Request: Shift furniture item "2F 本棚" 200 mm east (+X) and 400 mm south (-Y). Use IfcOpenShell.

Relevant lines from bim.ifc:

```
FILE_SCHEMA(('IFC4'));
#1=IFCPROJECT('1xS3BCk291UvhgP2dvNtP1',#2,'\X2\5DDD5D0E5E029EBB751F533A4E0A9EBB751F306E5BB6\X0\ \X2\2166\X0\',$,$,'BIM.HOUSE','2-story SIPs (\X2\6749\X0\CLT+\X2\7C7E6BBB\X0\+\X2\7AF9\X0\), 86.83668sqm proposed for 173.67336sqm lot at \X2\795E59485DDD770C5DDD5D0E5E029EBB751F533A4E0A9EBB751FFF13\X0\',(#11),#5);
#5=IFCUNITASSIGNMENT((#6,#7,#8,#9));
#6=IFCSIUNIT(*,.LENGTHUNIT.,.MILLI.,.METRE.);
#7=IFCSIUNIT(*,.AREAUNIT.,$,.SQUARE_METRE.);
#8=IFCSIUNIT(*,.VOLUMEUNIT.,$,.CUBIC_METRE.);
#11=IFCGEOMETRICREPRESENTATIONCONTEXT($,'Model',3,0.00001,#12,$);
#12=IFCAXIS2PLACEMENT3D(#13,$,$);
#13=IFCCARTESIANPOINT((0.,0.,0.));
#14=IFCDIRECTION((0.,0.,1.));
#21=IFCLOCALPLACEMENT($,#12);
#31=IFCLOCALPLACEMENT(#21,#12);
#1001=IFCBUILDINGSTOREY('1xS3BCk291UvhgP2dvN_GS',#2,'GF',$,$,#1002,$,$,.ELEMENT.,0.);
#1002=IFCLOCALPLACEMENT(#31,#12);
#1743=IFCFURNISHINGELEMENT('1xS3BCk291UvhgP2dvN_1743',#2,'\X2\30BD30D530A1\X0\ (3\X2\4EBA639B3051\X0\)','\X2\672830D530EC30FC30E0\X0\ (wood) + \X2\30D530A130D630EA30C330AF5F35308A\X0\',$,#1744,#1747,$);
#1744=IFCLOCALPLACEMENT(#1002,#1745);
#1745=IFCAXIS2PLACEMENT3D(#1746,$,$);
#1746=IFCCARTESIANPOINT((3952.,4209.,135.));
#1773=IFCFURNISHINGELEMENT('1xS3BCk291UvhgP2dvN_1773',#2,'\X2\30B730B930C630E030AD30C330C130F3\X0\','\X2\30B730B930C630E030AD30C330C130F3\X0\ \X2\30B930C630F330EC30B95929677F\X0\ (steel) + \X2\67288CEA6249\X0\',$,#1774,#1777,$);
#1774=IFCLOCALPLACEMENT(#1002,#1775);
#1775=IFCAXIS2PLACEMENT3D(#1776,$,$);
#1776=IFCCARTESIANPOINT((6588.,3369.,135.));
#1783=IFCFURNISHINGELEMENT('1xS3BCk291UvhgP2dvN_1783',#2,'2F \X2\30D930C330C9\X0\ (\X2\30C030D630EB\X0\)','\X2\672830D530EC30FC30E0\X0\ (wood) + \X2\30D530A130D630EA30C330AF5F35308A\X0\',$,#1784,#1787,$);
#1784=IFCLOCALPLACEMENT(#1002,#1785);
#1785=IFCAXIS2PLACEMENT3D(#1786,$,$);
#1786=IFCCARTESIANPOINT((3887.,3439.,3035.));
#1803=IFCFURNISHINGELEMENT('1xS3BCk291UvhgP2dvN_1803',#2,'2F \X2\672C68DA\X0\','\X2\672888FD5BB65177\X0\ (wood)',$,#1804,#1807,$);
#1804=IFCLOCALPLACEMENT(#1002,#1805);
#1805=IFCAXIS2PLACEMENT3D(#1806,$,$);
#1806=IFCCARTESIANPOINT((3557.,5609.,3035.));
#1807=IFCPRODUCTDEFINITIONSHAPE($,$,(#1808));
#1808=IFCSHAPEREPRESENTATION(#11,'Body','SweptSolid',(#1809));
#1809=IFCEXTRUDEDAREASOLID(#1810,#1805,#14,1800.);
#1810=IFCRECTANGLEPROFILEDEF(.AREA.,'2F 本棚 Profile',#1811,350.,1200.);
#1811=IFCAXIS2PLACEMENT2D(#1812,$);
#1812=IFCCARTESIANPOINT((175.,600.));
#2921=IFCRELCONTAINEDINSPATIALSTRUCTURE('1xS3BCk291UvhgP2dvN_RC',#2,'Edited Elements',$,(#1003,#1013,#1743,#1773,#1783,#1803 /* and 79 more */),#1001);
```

```python
import ifcopenshell
import ifcopenshell.api.geometry
import ifcopenshell.util.placement
import ifcopenshell.util.unit

model = ifcopenshell.open("bim.ifc")
unit_scale = ifcopenshell.util.unit.calculate_unit_scale(model)

item = model.by_guid("1xS3BCk291UvhgP2dvN_1803")
matrix = ifcopenshell.util.placement.get_local_placement(item.ObjectPlacement)
matrix[0, 3] += 0.2 / unit_scale
matrix[1, 3] -= 0.4 / unit_scale
ifcopenshell.api.geometry.edit_object_placement(model, product=item, matrix=matrix, is_si=False)

print(ifcopenshell.util.placement.get_local_placement(item.ObjectPlacement).round(3) + 0.0)

model.write("bim_updated.ifc")
```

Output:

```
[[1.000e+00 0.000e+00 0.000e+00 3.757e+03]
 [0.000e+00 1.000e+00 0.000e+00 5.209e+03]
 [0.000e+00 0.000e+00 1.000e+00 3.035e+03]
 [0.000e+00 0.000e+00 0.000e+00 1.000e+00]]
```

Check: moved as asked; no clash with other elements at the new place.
